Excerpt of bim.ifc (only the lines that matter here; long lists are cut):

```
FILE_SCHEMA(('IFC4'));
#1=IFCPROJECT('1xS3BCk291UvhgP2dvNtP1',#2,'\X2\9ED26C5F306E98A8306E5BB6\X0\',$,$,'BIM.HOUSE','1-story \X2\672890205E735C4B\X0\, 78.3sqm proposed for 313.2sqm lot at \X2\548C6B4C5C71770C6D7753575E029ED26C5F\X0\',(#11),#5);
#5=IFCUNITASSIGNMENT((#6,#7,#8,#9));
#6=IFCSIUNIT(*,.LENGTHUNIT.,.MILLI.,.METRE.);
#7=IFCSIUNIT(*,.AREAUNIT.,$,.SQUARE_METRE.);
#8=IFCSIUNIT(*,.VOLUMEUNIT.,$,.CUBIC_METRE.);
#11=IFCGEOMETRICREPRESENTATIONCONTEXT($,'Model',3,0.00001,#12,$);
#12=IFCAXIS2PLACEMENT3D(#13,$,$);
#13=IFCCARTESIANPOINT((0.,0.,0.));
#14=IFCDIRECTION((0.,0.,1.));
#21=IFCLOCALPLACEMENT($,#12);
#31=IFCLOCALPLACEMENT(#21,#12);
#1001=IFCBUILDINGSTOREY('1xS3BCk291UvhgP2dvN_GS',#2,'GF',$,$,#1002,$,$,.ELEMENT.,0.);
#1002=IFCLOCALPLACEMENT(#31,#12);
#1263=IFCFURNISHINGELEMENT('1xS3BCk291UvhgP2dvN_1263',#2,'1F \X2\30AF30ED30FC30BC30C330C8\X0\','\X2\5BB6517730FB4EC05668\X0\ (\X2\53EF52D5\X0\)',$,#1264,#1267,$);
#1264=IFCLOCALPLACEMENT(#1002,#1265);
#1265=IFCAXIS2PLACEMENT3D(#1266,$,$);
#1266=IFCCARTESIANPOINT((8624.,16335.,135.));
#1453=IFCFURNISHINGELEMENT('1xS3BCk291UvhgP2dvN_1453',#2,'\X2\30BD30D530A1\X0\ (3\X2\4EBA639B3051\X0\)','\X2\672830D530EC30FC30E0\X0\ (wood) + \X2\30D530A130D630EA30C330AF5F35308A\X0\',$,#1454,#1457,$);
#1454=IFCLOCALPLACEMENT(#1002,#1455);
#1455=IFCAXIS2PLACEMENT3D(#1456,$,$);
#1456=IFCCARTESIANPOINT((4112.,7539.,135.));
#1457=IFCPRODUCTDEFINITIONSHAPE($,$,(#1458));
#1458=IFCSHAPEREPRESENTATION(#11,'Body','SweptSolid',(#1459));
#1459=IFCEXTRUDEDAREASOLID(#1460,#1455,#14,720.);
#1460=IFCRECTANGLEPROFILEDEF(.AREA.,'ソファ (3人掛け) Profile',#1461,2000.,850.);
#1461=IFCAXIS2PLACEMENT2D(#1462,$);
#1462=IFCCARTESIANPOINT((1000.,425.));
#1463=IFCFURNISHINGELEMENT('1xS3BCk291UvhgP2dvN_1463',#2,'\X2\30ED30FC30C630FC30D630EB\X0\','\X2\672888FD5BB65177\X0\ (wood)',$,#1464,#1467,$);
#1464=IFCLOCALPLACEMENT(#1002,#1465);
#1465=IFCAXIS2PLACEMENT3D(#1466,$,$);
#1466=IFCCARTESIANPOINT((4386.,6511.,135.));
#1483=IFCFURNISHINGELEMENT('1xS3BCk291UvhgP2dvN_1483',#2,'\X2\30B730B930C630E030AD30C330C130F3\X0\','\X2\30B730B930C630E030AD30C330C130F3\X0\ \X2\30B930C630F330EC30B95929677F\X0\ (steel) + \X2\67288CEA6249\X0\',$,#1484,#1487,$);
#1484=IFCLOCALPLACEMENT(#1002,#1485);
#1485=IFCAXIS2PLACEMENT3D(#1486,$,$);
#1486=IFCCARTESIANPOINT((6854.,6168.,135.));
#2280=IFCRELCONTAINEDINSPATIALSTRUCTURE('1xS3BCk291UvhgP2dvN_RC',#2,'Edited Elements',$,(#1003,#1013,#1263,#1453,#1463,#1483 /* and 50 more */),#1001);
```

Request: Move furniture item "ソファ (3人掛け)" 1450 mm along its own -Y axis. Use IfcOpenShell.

```python
import ifcopenshell
import ifcopenshell.api.geometry
import ifcopenshell.util.placement
import ifcopenshell.util.unit

model = ifcopenshell.open("bim.ifc")
unit_scale = ifcopenshell.util.unit.calculate_unit_scale(model)

item = model.by_guid("1xS3BCk291UvhgP2dvN_1453")
matrix = ifcopenshell.util.placement.get_local_placement(item.ObjectPlacement)
matrix[:3, 3] -= matrix[:3, 1] * 1.45 / unit_scale
ifcopenshell.api.geometry.edit_object_placement(model, product=item, matrix=matrix, is_si=False)

print(ifcopenshell.util.placement.get_local_placement(item.ObjectPlacement).round(3) + 0.0)

model.write("bim_edited.ifc")
```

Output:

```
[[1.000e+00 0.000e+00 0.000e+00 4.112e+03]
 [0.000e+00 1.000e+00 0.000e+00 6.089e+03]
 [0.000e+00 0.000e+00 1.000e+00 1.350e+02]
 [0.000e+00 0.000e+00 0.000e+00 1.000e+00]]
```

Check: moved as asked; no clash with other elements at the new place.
